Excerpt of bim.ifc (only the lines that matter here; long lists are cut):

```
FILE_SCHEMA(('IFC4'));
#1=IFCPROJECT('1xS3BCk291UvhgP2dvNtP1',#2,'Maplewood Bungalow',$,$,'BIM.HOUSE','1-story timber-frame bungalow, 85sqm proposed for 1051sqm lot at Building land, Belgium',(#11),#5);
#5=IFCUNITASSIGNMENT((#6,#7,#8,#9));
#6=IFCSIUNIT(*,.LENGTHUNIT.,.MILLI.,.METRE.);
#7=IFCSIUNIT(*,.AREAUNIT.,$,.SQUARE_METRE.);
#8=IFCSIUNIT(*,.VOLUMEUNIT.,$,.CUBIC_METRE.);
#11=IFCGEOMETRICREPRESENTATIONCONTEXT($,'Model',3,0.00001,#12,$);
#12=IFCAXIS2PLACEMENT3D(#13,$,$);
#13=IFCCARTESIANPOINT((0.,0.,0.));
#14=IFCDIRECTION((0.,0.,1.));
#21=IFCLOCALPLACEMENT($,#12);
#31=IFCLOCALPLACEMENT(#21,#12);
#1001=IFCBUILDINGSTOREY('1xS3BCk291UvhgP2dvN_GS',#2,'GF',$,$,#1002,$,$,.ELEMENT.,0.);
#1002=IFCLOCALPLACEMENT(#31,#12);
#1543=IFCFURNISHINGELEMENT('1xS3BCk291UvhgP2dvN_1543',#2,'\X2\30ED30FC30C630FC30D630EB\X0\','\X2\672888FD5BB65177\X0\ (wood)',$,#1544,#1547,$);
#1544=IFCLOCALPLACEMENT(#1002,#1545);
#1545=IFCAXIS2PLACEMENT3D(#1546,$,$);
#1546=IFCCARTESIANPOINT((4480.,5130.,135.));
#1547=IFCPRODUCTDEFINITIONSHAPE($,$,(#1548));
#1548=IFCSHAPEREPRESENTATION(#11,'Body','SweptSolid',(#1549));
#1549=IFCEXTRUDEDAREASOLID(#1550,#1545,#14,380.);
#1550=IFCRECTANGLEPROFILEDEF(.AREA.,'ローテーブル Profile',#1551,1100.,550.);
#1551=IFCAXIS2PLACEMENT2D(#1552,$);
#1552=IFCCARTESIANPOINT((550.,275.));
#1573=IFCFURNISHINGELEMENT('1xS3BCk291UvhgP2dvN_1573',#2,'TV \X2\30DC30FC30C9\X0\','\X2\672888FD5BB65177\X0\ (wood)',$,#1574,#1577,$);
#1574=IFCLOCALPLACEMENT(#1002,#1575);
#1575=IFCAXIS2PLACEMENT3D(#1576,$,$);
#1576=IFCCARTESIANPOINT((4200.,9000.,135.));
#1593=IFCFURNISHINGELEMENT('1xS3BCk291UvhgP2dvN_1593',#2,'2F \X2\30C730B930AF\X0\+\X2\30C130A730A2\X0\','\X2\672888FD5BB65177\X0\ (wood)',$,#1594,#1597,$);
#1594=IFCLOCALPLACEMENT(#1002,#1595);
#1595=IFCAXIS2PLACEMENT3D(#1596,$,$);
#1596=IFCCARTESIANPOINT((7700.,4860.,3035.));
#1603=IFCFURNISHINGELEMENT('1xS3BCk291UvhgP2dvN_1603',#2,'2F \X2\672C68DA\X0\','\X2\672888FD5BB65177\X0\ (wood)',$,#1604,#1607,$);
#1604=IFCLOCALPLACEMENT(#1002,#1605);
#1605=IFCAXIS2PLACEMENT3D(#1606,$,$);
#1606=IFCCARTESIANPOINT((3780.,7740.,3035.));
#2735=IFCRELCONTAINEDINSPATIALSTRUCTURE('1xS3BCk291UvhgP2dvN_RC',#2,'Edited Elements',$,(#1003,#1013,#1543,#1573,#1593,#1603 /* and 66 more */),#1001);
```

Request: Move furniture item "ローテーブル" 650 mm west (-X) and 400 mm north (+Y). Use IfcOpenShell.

```python
import ifcopenshell
import ifcopenshell.api.geometry
import ifcopenshell.util.placement
import ifcopenshell.util.unit

model = ifcopenshell.open("bim.ifc")
unit_scale = ifcopenshell.util.unit.calculate_unit_scale(model)

item = model.by_id(1543)
matrix = ifcopenshell.util.placement.get_local_placement(item.ObjectPlacement)
matrix[0, 3] -= 0.65 / unit_scale
matrix[1, 3] += 0.4 / unit_scale
ifcopenshell.api.geometry.edit_object_placement(model, product=item, matrix=matrix, is_si=False)

print(ifcopenshell.util.placement.get_local_placement(item.ObjectPlacement).round(3) + 0.0)

model.write("bim_rev.ifc")
```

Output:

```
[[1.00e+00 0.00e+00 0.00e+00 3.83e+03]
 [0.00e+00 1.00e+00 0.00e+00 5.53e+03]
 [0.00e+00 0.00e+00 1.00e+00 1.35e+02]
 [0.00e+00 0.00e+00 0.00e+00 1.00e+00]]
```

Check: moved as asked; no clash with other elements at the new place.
